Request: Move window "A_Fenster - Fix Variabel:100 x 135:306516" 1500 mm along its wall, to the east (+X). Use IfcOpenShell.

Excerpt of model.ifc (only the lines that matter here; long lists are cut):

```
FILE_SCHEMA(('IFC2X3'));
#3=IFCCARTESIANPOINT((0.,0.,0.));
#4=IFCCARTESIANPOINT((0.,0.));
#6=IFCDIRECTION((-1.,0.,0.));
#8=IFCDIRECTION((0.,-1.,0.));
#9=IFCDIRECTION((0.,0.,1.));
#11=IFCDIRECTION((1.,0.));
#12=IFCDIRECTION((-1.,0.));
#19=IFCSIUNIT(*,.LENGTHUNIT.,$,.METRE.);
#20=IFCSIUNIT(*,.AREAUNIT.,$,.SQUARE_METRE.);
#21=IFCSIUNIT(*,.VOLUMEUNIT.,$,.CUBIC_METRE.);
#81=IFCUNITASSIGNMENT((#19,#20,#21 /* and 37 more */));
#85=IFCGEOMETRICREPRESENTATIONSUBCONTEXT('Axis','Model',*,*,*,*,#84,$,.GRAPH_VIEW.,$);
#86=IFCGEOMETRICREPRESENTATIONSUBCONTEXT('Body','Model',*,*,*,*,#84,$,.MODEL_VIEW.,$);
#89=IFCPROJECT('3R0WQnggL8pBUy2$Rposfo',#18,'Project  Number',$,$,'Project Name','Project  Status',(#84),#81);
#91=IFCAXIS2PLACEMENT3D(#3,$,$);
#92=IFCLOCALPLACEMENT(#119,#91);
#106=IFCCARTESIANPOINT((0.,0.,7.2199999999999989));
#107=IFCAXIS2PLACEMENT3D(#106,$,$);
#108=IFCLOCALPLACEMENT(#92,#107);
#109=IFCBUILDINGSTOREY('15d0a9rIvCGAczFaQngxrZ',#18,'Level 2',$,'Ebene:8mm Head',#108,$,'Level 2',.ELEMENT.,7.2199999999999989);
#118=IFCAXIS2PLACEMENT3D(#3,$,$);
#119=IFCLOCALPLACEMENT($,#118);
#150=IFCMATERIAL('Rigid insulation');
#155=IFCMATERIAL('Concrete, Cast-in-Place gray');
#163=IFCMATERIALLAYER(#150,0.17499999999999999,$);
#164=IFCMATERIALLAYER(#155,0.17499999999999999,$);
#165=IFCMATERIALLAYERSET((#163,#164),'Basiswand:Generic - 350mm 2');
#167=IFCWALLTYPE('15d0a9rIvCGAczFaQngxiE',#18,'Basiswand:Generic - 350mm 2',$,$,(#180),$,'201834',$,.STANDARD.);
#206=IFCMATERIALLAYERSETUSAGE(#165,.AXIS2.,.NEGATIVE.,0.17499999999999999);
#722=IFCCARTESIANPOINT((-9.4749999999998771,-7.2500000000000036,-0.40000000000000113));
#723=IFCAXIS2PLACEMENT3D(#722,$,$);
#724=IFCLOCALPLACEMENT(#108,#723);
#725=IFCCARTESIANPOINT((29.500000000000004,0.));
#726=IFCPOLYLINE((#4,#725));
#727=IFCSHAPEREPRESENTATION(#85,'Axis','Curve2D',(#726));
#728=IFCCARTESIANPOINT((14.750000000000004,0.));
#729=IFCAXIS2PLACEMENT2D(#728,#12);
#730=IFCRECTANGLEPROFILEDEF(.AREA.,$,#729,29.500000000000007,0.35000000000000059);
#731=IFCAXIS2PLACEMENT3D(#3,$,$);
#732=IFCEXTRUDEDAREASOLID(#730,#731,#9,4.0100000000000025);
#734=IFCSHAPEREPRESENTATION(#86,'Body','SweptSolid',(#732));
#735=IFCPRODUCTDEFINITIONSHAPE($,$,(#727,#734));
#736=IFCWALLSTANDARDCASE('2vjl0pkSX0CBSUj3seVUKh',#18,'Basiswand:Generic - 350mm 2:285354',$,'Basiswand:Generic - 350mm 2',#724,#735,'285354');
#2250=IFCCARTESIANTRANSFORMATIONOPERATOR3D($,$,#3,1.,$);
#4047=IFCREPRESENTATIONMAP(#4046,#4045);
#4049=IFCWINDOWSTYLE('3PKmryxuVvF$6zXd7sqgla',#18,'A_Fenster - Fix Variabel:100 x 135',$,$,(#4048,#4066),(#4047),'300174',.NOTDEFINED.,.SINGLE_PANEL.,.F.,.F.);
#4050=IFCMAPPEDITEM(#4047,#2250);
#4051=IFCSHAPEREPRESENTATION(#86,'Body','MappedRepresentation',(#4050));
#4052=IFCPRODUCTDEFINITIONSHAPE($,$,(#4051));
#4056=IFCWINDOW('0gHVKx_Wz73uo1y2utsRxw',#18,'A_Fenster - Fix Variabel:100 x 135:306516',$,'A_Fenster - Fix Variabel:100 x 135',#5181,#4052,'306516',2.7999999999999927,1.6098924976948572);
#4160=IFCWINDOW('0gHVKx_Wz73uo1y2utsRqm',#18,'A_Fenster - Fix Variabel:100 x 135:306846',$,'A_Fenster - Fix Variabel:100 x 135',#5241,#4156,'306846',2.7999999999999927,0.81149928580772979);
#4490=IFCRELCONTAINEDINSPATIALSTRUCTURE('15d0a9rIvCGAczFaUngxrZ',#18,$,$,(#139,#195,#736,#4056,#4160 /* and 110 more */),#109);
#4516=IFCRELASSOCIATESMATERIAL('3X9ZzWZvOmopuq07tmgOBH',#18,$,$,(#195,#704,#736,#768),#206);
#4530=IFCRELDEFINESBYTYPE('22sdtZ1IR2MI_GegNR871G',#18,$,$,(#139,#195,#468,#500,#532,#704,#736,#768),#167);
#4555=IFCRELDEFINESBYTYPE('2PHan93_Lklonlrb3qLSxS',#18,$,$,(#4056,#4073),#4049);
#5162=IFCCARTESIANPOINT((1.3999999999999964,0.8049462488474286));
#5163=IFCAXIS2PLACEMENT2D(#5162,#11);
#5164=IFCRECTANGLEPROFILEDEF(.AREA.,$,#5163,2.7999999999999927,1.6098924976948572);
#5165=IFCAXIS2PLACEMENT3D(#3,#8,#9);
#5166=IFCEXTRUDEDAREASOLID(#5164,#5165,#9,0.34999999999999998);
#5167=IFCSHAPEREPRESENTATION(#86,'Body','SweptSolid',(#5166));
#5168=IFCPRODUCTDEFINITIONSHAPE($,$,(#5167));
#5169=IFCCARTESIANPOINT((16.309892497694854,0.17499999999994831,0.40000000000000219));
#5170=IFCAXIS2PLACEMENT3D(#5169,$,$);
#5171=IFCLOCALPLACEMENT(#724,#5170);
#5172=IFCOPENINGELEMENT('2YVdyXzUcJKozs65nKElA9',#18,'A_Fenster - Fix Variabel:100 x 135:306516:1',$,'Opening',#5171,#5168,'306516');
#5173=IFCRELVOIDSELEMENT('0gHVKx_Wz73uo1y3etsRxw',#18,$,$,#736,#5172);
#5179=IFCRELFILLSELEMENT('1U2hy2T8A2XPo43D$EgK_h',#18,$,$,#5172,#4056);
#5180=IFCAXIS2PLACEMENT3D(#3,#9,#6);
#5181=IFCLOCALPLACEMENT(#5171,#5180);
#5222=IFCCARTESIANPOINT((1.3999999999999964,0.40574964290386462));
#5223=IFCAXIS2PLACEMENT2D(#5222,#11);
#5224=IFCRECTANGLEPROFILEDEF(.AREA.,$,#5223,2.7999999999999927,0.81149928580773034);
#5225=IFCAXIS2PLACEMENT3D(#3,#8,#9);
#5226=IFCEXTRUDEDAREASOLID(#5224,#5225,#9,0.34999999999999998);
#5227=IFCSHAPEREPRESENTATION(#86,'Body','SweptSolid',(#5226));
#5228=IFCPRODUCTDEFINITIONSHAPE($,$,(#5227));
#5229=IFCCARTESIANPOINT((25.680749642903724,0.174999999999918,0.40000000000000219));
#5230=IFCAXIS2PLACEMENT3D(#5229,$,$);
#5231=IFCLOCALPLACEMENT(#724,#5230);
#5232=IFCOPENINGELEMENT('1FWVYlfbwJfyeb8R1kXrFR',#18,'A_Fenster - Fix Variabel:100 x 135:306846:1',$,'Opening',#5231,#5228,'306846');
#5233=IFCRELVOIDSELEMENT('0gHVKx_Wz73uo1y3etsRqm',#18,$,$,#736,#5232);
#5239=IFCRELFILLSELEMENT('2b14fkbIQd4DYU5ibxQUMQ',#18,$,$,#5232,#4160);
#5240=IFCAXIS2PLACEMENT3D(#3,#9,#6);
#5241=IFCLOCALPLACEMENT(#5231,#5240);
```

```python
import ifcopenshell
import ifcopenshell.api.geometry
import ifcopenshell.util.placement
import ifcopenshell.util.unit

model = ifcopenshell.open("model.ifc")
unit_scale = ifcopenshell.util.unit.calculate_unit_scale(model)

window = model.by_guid("0gHVKx_Wz73uo1y2utsRxw")
opening = window.FillsVoids[0].RelatingOpeningElement
wall = opening.VoidsElements[0].RelatingBuildingElement

wall_matrix = ifcopenshell.util.placement.get_local_placement(wall.ObjectPlacement)
shift = wall_matrix[:3, 0] * 1.5 / unit_scale
before = ifcopenshell.util.placement.get_local_placement(window.ObjectPlacement)[:3, 3].copy()

# The window is placed relative to its opening, so it follows when the opening moves.
matrix = ifcopenshell.util.placement.get_local_placement(opening.ObjectPlacement)
matrix[:3, 3] += shift
ifcopenshell.api.geometry.edit_object_placement(
    model, product=opening, matrix=matrix, is_si=False, should_transform_children=True
)

after = ifcopenshell.util.placement.get_local_placement(window.ObjectPlacement)[:3, 3]
print("window moved by", (after - before).round(3) + 0.0)

model.write("model_rev.ifc")
```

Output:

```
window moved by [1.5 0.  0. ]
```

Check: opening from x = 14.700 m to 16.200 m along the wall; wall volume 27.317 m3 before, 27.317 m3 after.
